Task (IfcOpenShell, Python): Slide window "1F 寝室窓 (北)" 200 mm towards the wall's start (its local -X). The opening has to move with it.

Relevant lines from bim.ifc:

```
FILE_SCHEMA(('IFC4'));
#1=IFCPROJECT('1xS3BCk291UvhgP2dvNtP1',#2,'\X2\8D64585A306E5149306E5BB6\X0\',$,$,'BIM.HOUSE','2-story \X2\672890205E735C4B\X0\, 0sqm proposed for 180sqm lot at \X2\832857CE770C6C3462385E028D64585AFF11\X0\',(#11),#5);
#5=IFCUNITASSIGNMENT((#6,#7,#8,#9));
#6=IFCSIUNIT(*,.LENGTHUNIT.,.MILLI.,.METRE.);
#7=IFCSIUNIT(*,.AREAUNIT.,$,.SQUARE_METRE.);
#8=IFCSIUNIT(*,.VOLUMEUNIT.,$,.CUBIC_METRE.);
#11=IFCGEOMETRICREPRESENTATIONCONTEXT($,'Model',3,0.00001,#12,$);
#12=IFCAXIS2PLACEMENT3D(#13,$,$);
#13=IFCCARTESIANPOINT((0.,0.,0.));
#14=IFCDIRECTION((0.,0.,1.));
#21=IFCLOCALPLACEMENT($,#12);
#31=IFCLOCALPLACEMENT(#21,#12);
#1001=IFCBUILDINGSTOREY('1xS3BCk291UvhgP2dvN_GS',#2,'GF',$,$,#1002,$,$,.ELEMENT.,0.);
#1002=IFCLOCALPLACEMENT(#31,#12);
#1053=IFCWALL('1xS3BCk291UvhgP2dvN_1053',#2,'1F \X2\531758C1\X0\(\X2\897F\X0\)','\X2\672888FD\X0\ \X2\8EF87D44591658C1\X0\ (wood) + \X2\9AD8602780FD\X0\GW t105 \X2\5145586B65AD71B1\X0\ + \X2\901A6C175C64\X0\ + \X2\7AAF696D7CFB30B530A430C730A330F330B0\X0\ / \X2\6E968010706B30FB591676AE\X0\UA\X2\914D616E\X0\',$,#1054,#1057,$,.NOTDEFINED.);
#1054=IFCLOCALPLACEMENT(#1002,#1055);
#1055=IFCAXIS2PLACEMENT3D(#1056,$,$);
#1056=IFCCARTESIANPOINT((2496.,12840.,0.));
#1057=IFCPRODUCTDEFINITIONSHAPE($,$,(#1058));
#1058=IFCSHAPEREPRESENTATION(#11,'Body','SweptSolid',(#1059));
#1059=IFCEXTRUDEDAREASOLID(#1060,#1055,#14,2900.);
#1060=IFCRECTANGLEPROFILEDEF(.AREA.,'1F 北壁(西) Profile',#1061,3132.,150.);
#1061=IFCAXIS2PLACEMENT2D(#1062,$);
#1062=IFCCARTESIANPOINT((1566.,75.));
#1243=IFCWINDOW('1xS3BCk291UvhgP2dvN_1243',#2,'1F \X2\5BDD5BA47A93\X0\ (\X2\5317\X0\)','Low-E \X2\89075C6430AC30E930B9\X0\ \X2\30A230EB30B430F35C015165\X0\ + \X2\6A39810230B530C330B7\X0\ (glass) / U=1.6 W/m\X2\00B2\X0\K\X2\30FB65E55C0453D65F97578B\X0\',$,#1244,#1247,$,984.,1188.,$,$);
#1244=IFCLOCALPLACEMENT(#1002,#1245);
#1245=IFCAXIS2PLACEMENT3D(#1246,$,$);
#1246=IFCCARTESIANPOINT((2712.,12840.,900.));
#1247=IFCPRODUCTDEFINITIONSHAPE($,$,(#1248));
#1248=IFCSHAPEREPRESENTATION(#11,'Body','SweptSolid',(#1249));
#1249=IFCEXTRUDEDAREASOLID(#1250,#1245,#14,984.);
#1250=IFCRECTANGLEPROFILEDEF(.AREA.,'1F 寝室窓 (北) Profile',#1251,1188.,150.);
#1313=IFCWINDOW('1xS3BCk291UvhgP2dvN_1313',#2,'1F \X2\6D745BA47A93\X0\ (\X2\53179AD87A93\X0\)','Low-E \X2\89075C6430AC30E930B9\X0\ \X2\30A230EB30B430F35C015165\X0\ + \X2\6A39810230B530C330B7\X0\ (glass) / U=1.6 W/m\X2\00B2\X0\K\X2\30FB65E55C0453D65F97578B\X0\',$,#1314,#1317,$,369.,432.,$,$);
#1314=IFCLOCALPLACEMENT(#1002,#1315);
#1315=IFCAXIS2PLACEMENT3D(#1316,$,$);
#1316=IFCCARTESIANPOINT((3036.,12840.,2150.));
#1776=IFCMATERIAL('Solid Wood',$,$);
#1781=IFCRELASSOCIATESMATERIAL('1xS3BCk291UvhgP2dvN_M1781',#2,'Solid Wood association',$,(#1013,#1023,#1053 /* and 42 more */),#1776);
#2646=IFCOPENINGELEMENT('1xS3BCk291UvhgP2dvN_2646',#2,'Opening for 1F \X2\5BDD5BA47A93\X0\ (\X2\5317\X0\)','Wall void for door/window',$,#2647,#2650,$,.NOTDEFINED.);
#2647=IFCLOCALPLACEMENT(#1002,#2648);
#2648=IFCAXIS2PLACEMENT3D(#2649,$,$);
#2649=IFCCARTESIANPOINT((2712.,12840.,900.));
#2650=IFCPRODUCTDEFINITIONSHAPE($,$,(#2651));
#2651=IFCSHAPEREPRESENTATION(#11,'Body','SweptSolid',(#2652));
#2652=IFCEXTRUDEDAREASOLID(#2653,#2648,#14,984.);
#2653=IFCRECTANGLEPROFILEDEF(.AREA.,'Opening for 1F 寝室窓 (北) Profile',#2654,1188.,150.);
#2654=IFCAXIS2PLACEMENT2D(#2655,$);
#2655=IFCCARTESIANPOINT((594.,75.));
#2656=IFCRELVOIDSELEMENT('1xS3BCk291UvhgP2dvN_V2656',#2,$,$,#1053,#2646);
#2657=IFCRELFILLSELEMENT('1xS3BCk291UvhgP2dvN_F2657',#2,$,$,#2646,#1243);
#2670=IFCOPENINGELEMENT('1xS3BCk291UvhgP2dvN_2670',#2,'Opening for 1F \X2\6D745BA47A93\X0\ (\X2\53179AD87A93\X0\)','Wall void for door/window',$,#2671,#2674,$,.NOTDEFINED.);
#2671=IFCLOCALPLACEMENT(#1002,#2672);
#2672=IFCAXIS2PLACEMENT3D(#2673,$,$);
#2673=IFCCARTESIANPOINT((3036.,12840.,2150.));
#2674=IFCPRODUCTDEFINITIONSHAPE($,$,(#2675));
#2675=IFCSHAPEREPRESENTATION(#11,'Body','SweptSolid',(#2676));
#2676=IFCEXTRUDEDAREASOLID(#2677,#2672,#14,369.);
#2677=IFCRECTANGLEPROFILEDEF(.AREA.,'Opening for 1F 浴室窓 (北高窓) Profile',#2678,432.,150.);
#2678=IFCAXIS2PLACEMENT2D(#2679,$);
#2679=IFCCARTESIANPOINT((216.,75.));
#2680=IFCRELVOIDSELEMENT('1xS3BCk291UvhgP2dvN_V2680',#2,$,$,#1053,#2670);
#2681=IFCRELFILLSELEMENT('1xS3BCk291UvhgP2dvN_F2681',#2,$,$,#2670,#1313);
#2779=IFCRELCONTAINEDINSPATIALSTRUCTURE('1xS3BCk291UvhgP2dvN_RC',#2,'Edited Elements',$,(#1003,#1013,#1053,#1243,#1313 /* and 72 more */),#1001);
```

```python
import ifcopenshell
import ifcopenshell.api.geometry
import ifcopenshell.util.placement
import ifcopenshell.util.unit

model = ifcopenshell.open("bim.ifc")
unit_scale = ifcopenshell.util.unit.calculate_unit_scale(model)

window = model.by_guid("1xS3BCk291UvhgP2dvN_1243")
opening = window.FillsVoids[0].RelatingOpeningElement
wall = opening.VoidsElements[0].RelatingBuildingElement

wall_matrix = ifcopenshell.util.placement.get_local_placement(wall.ObjectPlacement)
shift = wall_matrix[:3, 0] * -0.2 / unit_scale
before = ifcopenshell.util.placement.get_local_placement(window.ObjectPlacement)[:3, 3].copy()

# The window is not placed relative to its opening, so move both.
for product in (opening, window):
    matrix = ifcopenshell.util.placement.get_local_placement(product.ObjectPlacement)
    matrix[:3, 3] += shift
    ifcopenshell.api.geometry.edit_object_placement(model, product=product, matrix=matrix, is_si=False)

after = ifcopenshell.util.placement.get_local_placement(window.ObjectPlacement)[:3, 3]
print("window moved by", (after - before).round(3) + 0.0)

model.write("bim_updated.ifc")
```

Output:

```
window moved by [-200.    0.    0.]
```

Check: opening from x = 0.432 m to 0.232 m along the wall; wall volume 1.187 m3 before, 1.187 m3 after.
